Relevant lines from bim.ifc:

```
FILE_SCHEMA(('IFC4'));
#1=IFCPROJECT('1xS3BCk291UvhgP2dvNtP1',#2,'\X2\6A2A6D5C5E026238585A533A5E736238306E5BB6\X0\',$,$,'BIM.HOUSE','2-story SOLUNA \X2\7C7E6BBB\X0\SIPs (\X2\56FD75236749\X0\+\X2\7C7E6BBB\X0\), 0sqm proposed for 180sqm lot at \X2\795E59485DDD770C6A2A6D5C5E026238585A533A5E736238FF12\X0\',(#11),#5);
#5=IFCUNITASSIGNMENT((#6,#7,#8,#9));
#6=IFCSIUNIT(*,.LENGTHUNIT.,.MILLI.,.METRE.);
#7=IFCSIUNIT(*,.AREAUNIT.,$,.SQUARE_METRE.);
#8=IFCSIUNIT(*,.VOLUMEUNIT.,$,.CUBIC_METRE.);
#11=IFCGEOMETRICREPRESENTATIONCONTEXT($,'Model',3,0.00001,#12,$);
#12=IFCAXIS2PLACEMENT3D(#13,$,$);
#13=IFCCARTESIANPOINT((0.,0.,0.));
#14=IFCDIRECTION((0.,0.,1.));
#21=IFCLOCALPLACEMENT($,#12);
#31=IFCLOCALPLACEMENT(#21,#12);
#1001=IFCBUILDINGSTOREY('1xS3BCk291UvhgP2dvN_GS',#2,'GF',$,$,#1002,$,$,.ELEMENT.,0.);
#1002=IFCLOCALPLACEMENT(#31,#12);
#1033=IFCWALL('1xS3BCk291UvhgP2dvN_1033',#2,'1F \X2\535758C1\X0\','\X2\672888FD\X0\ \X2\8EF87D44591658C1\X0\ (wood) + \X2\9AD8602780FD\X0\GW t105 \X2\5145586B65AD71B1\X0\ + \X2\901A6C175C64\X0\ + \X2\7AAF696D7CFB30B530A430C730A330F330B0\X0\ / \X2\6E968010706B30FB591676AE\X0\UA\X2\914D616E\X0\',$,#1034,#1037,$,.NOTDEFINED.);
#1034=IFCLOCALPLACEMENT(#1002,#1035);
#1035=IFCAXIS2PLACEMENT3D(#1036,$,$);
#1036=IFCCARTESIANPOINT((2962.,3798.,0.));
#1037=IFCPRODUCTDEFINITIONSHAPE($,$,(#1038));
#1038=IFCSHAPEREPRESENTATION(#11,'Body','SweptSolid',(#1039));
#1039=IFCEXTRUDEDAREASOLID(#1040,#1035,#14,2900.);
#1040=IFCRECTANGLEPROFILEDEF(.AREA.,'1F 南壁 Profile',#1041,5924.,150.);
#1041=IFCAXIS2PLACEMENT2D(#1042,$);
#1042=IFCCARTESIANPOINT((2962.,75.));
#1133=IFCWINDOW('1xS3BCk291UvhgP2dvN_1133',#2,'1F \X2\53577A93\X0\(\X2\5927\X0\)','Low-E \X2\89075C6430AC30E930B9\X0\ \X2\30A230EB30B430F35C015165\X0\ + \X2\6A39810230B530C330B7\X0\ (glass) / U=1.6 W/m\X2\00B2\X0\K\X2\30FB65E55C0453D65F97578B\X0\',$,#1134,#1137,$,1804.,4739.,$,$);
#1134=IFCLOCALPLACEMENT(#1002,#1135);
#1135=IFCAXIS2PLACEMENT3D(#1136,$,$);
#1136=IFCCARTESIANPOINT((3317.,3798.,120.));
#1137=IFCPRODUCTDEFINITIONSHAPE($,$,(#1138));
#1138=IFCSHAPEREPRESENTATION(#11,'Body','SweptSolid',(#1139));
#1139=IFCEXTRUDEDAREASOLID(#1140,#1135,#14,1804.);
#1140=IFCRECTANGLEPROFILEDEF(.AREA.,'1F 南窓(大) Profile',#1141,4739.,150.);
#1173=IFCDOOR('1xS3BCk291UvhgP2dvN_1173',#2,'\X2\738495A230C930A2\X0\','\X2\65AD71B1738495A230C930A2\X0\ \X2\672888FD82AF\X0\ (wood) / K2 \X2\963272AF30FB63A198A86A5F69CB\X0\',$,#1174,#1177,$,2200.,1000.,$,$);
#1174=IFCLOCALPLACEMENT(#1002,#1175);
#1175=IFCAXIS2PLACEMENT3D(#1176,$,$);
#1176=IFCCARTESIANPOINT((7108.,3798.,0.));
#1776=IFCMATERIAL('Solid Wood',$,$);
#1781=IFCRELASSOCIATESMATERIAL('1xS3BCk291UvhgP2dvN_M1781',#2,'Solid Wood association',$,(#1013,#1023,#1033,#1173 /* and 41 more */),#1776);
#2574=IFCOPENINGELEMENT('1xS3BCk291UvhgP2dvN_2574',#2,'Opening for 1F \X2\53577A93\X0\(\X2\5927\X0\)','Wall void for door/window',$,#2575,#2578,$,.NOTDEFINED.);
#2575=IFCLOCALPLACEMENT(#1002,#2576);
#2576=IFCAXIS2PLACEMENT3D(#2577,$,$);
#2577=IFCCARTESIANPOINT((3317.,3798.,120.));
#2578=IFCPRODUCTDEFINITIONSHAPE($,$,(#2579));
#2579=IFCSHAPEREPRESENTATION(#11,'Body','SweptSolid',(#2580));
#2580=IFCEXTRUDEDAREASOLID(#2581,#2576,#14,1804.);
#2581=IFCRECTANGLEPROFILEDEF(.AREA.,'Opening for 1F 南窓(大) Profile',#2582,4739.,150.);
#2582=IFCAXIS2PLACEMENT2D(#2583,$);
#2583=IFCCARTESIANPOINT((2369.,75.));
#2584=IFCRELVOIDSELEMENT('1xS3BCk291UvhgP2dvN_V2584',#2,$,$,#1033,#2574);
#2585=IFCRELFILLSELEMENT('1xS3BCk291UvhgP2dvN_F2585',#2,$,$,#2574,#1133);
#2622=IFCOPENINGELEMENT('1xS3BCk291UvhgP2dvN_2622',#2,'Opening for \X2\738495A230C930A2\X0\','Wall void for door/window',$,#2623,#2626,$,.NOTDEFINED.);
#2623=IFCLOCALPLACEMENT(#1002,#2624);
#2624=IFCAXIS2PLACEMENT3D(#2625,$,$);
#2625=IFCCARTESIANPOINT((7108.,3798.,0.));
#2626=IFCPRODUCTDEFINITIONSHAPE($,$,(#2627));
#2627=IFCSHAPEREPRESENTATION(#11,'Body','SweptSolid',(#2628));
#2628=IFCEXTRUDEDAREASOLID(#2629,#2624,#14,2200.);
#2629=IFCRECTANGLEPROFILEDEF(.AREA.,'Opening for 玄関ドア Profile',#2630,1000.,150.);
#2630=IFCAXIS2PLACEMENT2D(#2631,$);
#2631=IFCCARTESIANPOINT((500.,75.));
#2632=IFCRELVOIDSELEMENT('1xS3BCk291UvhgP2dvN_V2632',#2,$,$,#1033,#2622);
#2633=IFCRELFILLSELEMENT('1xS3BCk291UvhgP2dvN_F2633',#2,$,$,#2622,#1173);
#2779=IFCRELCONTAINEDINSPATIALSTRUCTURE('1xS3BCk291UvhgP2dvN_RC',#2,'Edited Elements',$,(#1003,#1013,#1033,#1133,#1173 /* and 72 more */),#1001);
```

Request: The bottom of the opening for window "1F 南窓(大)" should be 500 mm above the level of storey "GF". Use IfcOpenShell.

```python
import numpy as np
import ifcopenshell
import ifcopenshell.api.geometry
import ifcopenshell.geom
import ifcopenshell.util.element
import ifcopenshell.util.placement
import ifcopenshell.util.shape
import ifcopenshell.util.unit

model = ifcopenshell.open("bim.ifc")
unit_scale = ifcopenshell.util.unit.calculate_unit_scale(model)

window = model.by_id(1133)
opening = window.FillsVoids[0].RelatingOpeningElement
storey = ifcopenshell.util.element.get_container(window, ifc_class="IfcBuildingStorey")
level = ifcopenshell.util.placement.get_local_placement(storey.ObjectPlacement)[2, 3]

# The opening's origin need not be at the sill, so measure its lowest point.
shape = ifcopenshell.geom.create_shape(ifcopenshell.geom.settings(), opening)
bottom = ifcopenshell.util.shape.get_shape_bottom_elevation(shape, shape.geometry) / unit_scale
dz = level + 0.5 / unit_scale - bottom

shift = np.array([0.0, 0.0, dz])
# The window is not placed relative to its opening, so move both.
for product in (opening, window):
    matrix = ifcopenshell.util.placement.get_local_placement(product.ObjectPlacement)
    matrix[:3, 3] += shift
    ifcopenshell.api.geometry.edit_object_placement(model, product=product, matrix=matrix, is_si=False)

print(f"moved by {dz * unit_scale:+.3f} m")

model.write("bim_rev.ifc")
```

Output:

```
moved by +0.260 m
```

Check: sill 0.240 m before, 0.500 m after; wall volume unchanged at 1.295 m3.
